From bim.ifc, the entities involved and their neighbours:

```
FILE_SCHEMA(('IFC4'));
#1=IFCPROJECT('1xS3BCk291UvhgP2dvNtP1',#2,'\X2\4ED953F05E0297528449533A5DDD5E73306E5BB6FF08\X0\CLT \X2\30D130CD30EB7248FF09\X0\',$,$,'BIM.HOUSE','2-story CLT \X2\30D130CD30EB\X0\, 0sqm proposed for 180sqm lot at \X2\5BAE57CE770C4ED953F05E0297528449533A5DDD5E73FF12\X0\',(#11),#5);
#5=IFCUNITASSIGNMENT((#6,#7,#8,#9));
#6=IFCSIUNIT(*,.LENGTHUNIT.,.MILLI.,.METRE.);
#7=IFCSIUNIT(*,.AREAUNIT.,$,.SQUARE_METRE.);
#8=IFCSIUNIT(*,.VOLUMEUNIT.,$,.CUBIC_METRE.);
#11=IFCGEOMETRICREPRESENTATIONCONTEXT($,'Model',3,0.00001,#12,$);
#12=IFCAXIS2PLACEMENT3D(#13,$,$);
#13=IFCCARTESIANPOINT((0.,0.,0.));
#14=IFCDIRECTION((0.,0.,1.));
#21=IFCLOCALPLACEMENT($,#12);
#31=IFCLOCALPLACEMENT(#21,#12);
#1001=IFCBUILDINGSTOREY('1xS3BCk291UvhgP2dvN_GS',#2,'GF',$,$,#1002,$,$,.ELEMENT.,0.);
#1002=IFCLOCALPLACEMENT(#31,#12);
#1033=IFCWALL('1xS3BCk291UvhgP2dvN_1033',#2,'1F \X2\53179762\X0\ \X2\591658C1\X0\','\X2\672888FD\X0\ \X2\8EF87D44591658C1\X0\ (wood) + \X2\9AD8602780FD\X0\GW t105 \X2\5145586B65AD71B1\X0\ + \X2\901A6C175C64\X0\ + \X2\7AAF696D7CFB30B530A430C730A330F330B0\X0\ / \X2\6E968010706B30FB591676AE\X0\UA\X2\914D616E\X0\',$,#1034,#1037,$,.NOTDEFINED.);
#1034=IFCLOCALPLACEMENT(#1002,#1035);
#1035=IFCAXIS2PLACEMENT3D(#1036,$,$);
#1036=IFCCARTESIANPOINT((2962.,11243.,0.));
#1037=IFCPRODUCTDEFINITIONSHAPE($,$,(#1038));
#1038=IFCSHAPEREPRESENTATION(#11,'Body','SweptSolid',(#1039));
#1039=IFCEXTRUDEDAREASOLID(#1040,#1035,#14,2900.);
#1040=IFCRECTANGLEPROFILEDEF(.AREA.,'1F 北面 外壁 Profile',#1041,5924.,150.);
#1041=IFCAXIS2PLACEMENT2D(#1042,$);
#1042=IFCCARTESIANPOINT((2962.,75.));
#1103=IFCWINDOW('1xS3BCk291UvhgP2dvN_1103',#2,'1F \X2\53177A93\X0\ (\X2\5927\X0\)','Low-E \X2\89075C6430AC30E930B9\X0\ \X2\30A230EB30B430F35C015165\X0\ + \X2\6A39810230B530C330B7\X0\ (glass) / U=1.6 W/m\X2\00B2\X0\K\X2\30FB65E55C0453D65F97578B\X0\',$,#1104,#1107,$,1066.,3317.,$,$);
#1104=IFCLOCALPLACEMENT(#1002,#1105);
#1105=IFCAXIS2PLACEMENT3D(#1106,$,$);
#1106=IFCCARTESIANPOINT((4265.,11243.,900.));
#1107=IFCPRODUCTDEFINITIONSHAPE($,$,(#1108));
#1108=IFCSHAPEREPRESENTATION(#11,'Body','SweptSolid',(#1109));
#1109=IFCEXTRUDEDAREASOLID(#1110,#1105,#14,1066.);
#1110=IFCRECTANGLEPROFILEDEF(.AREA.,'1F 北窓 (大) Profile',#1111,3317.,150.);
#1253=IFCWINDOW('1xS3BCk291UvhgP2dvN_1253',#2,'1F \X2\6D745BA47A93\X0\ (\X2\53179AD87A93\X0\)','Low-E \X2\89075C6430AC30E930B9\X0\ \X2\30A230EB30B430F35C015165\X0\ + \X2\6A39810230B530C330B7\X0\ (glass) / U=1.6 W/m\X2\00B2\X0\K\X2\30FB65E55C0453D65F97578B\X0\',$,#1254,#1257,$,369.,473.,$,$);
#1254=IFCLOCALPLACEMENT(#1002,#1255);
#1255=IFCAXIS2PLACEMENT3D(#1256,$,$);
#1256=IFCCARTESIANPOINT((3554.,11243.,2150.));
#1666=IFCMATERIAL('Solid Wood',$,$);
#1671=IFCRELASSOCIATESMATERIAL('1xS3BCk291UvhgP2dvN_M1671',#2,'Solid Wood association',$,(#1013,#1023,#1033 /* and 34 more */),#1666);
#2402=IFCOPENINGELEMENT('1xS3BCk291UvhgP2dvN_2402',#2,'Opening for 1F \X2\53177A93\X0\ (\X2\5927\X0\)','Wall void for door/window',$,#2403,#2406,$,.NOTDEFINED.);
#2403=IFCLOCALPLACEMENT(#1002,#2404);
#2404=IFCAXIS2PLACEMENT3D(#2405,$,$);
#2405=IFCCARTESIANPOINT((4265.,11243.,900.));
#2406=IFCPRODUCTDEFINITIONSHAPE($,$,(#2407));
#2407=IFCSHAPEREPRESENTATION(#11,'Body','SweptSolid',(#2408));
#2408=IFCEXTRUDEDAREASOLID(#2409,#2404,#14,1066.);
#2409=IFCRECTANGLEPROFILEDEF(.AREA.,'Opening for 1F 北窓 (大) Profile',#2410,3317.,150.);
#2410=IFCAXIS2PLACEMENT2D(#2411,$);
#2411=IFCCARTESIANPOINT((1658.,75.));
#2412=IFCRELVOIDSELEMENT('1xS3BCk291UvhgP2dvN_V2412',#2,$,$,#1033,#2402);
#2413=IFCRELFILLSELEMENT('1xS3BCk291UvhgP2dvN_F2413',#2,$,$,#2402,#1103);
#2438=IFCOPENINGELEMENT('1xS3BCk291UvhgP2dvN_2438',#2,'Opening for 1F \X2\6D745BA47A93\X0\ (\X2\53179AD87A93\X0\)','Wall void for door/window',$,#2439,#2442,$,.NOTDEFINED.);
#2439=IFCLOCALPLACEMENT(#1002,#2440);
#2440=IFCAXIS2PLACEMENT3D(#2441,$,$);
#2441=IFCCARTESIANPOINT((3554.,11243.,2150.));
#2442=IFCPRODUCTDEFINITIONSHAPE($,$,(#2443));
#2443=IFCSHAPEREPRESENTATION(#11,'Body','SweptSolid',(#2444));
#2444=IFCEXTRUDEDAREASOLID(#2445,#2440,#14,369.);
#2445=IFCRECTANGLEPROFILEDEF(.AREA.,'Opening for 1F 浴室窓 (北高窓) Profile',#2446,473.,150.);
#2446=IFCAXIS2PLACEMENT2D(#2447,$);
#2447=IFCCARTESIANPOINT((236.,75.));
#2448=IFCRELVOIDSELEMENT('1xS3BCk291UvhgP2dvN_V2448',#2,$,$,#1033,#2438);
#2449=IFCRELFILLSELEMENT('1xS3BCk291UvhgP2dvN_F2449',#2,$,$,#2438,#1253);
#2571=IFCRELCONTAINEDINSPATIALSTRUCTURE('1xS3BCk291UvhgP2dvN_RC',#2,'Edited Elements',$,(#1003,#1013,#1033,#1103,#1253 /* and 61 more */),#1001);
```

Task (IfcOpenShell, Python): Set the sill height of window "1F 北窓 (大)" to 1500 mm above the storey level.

```python
import numpy as np
import ifcopenshell
import ifcopenshell.api.geometry
import ifcopenshell.geom
import ifcopenshell.util.element
import ifcopenshell.util.placement
import ifcopenshell.util.shape
import ifcopenshell.util.unit

model = ifcopenshell.open("bim.ifc")
unit_scale = ifcopenshell.util.unit.calculate_unit_scale(model)

window = model.by_guid("1xS3BCk291UvhgP2dvN_1103")
opening = window.FillsVoids[0].RelatingOpeningElement
storey = ifcopenshell.util.element.get_container(window, ifc_class="IfcBuildingStorey")
level = ifcopenshell.util.placement.get_local_placement(storey.ObjectPlacement)[2, 3]

# The opening's origin need not be at the sill, so measure its lowest point.
shape = ifcopenshell.geom.create_shape(ifcopenshell.geom.settings(), opening)
bottom = ifcopenshell.util.shape.get_shape_bottom_elevation(shape, shape.geometry) / unit_scale
dz = level + 1.5 / unit_scale - bottom

shift = np.array([0.0, 0.0, dz])
# The window is not placed relative to its opening, so move both.
for product in (opening, window):
    matrix = ifcopenshell.util.placement.get_local_placement(product.ObjectPlacement)
    matrix[:3, 3] += shift
    ifcopenshell.api.geometry.edit_object_placement(model, product=product, matrix=matrix, is_si=False)

print(f"moved by {dz * unit_scale:+.3f} m")

model.write("bim_rev.ifc")
```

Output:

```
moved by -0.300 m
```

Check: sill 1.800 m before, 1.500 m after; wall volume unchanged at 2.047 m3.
